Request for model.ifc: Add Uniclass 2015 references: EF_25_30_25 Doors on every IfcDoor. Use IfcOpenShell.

First a look at what the model holds.

```python
import ifcopenshell

model = ifcopenshell.open("model.ifc")
print(model.schema)
print("classifications:", [c.Name for c in model.by_type("IfcClassification")])
for ifc_class in ("IfcDoor", "IfcRoof", "IfcStair", "IfcWall", "IfcWindow"):
    print(ifc_class, len(model.by_type(ifc_class)))
```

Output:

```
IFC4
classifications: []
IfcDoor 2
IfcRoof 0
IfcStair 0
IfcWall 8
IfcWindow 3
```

```python
import ifcopenshell
import ifcopenshell.api.classification

model = ifcopenshell.open("model.ifc")

system = ifcopenshell.api.classification.add_classification(model, classification="Uniclass 2015")

codes = {
    "IfcDoor": ("EF_25_30_25", "Doors"),
}
for ifc_class, (code, name) in codes.items():
    products = model.by_type(ifc_class)
    ifcopenshell.api.classification.add_reference(
        model, products=products, classification=system, identification=code, name=name
    )
    print(code, len(products))

model.write("model-out.ifc")
```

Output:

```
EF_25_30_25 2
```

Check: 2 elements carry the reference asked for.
